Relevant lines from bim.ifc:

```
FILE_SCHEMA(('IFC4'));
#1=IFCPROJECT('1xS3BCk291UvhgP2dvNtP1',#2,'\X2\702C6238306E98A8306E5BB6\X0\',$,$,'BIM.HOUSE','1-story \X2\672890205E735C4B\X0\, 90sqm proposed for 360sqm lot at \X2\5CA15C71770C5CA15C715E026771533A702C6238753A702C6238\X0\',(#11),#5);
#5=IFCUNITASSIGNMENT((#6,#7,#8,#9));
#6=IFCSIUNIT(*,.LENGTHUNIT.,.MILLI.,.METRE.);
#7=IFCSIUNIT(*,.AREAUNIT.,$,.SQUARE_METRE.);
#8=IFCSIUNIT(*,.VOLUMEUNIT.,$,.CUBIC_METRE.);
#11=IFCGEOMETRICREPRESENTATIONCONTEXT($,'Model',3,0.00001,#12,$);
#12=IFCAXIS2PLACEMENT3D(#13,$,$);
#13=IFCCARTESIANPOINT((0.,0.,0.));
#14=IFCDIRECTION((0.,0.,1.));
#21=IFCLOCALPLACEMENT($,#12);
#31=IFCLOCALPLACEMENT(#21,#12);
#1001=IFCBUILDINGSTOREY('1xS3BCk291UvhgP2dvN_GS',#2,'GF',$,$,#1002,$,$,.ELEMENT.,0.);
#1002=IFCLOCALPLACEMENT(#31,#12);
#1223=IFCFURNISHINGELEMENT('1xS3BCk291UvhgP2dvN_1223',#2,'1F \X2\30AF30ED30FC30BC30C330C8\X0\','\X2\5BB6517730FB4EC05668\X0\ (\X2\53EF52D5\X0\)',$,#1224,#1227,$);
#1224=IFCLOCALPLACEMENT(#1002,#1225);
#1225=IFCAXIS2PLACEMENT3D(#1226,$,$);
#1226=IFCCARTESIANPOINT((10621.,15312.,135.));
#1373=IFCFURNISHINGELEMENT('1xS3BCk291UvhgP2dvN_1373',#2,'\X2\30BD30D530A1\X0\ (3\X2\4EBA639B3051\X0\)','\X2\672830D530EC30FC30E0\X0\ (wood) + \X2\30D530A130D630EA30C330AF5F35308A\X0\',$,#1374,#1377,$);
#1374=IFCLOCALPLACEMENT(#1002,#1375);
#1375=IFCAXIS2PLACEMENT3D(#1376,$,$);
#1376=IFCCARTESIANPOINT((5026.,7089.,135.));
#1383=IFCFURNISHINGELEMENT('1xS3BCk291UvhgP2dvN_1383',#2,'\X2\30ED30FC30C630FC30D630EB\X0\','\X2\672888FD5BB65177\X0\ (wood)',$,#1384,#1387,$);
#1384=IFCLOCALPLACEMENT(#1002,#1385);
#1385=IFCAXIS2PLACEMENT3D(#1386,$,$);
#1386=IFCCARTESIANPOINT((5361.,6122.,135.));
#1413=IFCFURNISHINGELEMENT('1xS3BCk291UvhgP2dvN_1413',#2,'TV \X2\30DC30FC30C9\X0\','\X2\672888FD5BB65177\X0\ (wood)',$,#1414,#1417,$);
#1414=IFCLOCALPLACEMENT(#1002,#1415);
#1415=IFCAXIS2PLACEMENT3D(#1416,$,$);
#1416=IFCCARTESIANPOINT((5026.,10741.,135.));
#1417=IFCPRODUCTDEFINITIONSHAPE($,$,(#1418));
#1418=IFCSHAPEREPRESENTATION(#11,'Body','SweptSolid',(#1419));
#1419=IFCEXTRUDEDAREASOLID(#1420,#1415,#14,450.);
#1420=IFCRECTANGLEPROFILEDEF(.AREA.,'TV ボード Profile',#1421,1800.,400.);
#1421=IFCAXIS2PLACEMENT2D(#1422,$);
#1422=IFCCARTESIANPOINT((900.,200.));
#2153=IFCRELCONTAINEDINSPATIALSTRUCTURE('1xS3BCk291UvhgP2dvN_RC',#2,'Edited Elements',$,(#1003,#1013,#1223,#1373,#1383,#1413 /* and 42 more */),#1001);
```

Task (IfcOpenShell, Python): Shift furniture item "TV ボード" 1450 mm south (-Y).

```python
import ifcopenshell
import ifcopenshell.api.geometry
import ifcopenshell.util.placement

model = ifcopenshell.open("bim.ifc")

item = model.by_guid("1xS3BCk291UvhgP2dvN_1413")
matrix = ifcopenshell.util.placement.get_local_placement(item.ObjectPlacement)
matrix[1, 3] -= 1450.0
ifcopenshell.api.geometry.edit_object_placement(model, product=item, matrix=matrix, is_si=False)

print(ifcopenshell.util.placement.get_local_placement(item.ObjectPlacement).round(3) + 0.0)

model.write("bim_updated.ifc")
```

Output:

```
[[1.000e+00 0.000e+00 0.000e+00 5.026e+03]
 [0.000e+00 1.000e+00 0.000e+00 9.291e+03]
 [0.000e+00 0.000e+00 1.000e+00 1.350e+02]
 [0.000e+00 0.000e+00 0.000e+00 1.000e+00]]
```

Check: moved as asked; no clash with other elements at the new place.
